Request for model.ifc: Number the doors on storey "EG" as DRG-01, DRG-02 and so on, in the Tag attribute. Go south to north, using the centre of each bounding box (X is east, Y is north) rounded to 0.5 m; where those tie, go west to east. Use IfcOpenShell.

First a look at what the model holds.

```python
import ifcopenshell
import ifcopenshell.util.element
import ifcopenshell.util.placement

model = ifcopenshell.open("model.ifc")
print(model.schema)
storey = next(s for s in model.by_type("IfcBuildingStorey") if s.Name == "EG")
doors = [e for e in ifcopenshell.util.element.get_decomposition(storey) if e.is_a("IfcDoor")]
for e in sorted(doors, key=lambda e: e.id()):
    origin = ifcopenshell.util.placement.get_local_placement(e.ObjectPlacement)[:3, 3]
    print(e.id(), e.Tag, e.Name, origin.round(2) + 0.0, sep=" | ")
```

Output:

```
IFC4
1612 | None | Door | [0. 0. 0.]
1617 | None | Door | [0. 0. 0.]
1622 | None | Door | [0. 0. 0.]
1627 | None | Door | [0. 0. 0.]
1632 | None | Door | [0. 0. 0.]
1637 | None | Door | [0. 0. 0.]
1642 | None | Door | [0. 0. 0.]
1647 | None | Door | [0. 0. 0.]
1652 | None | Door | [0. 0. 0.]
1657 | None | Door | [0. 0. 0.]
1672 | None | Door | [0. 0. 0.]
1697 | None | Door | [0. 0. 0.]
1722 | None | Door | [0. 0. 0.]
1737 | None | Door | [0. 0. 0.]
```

```python
import ifcopenshell
import ifcopenshell.geom
import ifcopenshell.util.element
import ifcopenshell.util.shape

model = ifcopenshell.open("model.ifc")
settings = ifcopenshell.geom.settings()
settings.set("use-world-coords", True)


def centre(element):
    shape = ifcopenshell.geom.create_shape(settings, element)
    return ifcopenshell.util.shape.get_bbox_centroid(shape.geometry)


storey = next(s for s in model.by_type("IfcBuildingStorey") if s.Name == "EG")
doors = [e for e in ifcopenshell.util.element.get_decomposition(storey) if e.is_a("IfcDoor")]

# Insertion points can sit at a corner or the storey origin, so sort by the geometry (in metres).
centres = {e: centre(e) for e in doors}
doors.sort(key=lambda e: (round(centres[e][1] / 0.5), centres[e][0]))

for i, e in enumerate(doors, start=1):
    number = f"DRG-{i:02d}"
    e.Tag = number
    print(e.id(), number)

model.write("model_rev.ifc")
```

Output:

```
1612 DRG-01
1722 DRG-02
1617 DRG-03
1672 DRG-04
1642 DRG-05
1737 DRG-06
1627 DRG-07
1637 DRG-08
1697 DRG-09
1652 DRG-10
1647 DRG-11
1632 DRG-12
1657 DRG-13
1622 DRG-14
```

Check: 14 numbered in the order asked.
